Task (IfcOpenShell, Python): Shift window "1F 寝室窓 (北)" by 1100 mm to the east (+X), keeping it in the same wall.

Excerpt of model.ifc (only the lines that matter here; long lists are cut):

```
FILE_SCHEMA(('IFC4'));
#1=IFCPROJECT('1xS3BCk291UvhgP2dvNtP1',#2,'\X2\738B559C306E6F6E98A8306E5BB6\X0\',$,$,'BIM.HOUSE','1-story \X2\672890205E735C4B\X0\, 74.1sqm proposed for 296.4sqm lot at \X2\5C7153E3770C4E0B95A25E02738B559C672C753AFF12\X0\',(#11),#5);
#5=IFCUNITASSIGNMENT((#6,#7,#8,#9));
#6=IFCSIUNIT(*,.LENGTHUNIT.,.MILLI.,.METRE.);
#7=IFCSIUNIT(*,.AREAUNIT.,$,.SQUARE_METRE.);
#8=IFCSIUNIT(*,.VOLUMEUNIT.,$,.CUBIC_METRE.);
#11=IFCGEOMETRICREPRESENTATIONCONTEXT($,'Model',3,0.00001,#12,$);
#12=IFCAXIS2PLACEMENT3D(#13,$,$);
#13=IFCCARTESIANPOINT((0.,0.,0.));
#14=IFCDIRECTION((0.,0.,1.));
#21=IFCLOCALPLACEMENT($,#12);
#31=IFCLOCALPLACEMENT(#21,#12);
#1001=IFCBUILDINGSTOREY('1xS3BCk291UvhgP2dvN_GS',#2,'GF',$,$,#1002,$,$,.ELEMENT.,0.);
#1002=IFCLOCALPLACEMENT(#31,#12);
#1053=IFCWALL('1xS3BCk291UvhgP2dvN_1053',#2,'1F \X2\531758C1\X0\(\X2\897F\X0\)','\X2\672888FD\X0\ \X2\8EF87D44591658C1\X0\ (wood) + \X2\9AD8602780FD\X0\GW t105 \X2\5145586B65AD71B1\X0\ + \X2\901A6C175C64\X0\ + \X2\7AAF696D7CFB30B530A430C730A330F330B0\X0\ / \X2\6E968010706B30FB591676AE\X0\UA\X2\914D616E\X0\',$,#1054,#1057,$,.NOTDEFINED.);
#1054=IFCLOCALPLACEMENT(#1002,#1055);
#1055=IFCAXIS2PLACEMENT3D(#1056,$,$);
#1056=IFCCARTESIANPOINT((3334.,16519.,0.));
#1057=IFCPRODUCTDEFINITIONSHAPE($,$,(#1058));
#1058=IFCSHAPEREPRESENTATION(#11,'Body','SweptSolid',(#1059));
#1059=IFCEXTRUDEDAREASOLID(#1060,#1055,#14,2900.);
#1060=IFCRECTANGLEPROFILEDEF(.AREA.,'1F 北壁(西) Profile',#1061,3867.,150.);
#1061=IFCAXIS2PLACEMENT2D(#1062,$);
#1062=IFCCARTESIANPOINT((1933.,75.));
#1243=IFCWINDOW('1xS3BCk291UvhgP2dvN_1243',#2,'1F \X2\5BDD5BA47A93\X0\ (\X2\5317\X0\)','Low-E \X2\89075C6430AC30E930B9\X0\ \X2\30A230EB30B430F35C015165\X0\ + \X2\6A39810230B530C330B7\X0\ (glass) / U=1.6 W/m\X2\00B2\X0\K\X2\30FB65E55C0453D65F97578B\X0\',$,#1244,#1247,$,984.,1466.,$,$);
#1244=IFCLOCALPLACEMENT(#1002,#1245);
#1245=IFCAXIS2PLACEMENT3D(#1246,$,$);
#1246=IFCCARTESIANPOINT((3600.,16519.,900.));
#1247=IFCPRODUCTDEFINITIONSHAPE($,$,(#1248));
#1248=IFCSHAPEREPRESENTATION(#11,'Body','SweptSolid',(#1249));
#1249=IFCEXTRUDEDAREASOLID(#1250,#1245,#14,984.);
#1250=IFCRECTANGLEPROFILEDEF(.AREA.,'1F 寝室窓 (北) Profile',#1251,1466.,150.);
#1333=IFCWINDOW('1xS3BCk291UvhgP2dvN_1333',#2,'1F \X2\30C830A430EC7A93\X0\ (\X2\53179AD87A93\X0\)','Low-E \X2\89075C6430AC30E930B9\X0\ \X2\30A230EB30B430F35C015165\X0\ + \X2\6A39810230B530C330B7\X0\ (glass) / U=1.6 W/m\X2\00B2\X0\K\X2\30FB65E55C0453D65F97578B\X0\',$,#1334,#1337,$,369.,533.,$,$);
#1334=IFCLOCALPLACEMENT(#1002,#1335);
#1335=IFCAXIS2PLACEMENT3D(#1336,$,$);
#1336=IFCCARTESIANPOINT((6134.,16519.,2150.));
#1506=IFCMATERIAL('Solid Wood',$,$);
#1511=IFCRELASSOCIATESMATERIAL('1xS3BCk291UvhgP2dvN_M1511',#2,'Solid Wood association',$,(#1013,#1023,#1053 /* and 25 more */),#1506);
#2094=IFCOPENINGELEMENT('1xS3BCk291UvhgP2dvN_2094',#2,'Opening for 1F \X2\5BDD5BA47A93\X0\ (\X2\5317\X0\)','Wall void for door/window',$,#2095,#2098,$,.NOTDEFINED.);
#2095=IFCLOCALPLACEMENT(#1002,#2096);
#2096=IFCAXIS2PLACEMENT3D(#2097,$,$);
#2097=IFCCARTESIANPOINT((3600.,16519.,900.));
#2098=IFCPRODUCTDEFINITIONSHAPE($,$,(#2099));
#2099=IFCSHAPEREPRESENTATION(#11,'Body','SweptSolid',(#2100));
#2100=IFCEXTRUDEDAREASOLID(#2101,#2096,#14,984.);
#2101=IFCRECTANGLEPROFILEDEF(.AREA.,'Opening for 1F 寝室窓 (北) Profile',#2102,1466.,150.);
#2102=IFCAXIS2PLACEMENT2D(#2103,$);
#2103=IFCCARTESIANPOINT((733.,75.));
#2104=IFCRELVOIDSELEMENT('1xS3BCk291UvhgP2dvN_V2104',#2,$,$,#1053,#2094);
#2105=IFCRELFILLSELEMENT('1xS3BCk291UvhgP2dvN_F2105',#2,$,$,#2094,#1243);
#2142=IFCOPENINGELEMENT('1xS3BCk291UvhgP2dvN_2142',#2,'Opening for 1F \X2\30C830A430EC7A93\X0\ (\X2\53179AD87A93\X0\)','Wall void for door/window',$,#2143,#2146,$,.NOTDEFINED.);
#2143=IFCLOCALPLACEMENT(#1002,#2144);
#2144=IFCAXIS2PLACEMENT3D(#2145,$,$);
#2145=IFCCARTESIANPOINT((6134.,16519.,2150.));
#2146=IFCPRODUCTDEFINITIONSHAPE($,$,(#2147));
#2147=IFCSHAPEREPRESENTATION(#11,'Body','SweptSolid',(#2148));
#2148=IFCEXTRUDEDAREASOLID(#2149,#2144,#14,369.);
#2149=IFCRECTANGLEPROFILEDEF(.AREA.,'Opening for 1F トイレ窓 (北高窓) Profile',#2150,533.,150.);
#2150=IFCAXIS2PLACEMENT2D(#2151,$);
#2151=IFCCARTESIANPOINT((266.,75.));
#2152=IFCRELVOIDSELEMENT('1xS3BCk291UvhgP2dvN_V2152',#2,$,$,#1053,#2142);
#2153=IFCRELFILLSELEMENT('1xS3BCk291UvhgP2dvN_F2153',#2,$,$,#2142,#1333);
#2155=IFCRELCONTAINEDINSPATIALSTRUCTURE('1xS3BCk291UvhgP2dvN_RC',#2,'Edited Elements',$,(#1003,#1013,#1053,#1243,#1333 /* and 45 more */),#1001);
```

```python
import ifcopenshell
import ifcopenshell.api.geometry
import ifcopenshell.util.placement
import ifcopenshell.util.unit

model = ifcopenshell.open("model.ifc")
unit_scale = ifcopenshell.util.unit.calculate_unit_scale(model)

window = model.by_id(1243)
opening = window.FillsVoids[0].RelatingOpeningElement
wall = opening.VoidsElements[0].RelatingBuildingElement

wall_matrix = ifcopenshell.util.placement.get_local_placement(wall.ObjectPlacement)
shift = wall_matrix[:3, 0] * 1.1 / unit_scale
before = ifcopenshell.util.placement.get_local_placement(window.ObjectPlacement)[:3, 3].copy()

# The window is not placed relative to its opening, so move both.
for product in (opening, window):
    matrix = ifcopenshell.util.placement.get_local_placement(product.ObjectPlacement)
    matrix[:3, 3] += shift
    ifcopenshell.api.geometry.edit_object_placement(model, product=product, matrix=matrix, is_si=False)

after = ifcopenshell.util.placement.get_local_placement(window.ObjectPlacement)[:3, 3]
print("window moved by", (after - before).round(3) + 0.0)

model.write("model_v2.ifc")
```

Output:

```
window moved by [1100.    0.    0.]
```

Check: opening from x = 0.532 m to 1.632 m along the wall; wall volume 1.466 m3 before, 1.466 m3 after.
